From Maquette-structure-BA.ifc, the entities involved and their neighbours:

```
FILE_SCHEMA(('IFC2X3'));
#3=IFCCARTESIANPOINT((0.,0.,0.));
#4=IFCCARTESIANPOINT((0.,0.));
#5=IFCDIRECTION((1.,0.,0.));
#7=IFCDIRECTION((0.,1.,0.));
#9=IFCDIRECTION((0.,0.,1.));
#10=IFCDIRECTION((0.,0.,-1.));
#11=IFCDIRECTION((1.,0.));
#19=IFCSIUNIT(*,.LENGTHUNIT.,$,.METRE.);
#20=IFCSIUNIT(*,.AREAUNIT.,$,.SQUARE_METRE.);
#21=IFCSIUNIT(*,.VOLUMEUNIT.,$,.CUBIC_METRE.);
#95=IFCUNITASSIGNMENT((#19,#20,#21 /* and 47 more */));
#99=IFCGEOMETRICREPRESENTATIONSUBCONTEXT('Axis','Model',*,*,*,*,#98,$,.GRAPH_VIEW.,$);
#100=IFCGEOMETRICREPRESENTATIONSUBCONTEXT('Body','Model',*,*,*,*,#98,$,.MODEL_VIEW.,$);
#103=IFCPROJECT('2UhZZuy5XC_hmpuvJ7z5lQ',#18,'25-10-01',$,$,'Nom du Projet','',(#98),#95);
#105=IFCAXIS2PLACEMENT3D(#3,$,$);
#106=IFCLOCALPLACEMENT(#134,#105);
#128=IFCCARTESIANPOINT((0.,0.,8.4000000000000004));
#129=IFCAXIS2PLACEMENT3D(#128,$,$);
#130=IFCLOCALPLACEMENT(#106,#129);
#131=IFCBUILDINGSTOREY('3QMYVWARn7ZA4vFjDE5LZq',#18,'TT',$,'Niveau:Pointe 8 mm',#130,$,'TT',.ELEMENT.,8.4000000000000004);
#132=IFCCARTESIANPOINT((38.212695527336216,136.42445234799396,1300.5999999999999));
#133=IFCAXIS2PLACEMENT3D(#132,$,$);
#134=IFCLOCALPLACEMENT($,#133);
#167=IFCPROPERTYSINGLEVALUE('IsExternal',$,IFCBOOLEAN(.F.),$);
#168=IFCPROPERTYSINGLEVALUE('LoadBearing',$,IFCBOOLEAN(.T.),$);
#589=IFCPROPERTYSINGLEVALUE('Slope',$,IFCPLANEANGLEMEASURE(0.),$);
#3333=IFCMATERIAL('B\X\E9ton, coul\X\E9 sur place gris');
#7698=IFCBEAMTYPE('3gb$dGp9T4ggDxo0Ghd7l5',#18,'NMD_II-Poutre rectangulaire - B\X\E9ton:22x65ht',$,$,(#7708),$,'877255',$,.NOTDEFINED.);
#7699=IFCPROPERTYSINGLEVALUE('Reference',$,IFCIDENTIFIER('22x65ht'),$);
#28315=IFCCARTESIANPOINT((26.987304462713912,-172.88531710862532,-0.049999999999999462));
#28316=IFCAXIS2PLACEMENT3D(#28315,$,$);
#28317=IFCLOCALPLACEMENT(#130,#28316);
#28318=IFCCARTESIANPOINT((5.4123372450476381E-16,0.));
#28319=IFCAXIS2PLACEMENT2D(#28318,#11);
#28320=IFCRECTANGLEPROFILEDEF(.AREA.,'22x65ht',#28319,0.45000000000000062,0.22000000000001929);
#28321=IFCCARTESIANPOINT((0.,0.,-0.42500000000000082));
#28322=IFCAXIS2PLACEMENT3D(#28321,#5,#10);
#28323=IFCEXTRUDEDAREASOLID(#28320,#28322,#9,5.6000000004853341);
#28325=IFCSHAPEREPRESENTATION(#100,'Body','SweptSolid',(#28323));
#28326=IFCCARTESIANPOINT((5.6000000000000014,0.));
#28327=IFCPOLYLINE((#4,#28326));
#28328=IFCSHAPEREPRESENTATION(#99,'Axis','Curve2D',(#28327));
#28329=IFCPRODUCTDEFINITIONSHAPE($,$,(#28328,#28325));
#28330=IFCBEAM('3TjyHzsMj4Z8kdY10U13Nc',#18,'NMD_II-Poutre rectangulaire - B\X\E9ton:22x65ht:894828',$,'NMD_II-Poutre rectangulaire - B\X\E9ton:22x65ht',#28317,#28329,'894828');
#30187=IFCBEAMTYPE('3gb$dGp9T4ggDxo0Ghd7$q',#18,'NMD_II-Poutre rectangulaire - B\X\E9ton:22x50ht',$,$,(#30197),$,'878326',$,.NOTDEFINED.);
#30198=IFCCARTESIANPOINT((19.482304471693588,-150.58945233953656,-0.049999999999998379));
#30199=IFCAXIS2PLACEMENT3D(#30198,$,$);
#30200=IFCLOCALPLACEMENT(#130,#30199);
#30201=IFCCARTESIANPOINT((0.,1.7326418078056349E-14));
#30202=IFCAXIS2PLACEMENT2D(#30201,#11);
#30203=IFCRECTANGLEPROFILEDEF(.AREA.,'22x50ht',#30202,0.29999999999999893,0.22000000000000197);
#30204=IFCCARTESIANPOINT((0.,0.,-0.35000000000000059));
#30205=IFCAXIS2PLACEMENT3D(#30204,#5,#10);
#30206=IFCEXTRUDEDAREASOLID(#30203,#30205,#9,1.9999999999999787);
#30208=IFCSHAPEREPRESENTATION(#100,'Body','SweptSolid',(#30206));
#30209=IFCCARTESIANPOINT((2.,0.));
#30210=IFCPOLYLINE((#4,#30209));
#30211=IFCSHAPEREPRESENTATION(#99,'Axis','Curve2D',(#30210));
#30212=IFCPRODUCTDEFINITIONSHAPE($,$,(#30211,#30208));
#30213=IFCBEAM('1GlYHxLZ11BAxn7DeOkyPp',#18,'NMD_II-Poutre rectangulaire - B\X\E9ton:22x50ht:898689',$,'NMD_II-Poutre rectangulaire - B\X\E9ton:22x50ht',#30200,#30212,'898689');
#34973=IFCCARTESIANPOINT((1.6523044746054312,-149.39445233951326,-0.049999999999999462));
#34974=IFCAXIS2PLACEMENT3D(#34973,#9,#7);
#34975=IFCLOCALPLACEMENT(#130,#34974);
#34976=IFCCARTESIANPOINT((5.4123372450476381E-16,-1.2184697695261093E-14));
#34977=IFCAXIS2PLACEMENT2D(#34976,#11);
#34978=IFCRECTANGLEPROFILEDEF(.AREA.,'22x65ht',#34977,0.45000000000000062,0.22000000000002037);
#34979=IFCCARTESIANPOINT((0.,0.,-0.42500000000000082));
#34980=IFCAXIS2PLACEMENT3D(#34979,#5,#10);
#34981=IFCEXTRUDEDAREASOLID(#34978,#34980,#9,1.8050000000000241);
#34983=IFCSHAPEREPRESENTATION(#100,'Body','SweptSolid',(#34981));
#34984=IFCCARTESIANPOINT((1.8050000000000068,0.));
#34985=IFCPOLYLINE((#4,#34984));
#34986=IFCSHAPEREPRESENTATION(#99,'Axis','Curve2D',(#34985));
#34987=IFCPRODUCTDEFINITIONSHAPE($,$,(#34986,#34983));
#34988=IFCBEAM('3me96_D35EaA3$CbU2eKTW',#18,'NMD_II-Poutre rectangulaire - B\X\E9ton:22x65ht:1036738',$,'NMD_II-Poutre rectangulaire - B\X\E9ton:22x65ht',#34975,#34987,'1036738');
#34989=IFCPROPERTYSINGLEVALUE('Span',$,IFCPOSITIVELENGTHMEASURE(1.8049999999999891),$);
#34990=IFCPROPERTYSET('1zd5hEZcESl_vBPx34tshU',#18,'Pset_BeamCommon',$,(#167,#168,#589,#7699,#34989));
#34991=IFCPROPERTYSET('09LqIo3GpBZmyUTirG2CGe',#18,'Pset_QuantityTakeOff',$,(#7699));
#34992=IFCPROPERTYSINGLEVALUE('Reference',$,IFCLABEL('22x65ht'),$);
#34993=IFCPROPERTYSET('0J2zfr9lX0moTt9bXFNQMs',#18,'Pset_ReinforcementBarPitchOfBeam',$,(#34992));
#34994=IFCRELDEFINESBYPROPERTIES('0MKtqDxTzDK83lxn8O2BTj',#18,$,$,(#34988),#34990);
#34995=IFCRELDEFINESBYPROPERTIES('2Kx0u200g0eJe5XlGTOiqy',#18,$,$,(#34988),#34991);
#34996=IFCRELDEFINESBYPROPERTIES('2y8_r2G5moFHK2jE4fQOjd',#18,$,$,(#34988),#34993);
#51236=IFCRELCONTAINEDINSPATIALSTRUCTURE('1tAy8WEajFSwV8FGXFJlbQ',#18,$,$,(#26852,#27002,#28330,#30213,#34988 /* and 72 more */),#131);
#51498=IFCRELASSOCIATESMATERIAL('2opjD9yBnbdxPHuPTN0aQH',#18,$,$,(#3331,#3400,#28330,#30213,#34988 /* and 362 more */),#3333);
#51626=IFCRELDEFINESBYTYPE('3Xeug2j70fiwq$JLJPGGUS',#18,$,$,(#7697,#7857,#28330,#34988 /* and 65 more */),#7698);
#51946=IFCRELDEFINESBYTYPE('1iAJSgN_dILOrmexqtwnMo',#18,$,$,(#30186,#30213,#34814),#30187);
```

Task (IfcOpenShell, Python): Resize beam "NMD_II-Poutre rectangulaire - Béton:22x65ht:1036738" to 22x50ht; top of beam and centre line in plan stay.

```python
import ifcopenshell
import ifcopenshell.api.pset
import ifcopenshell.api.type
import ifcopenshell.util.element
import ifcopenshell.util.representation

model = ifcopenshell.open("Maquette-structure-BA.ifc")

member = model.by_id(34988)
source = next(p for p in model.by_type("IfcRectangleProfileDef") if p.ProfileName == "22x50ht")

body = ifcopenshell.util.representation.get_representation(member, "Model", "Body")
solid = body.Items[0]
old_profile = solid.SweptArea

# Copy the section's sizes but keep this member's own profile position.
profile = ifcopenshell.util.element.copy(model, source)
# Profiles are centred, so shift by half the change in depth to hold the top.
shift = (old_profile.XDim - profile.XDim) / 2
x, y = old_profile.Position.Location.Coordinates
up = (-1.0, 0.0)  # upwards, in the solid's own plane
location = model.createIfcCartesianPoint((x + up[0] * shift, y + up[1] * shift))
profile.Position = model.createIfcAxis2Placement2D(location, old_profile.Position.RefDirection)
solid.SweptArea = profile
if not model.get_total_inverses(old_profile):
    ifcopenshell.util.element.remove_deep2(model, old_profile)

new_type = model.by_guid("3gb$dGp9T4ggDxo0Ghd7$q")
ifcopenshell.api.type.assign_type(
    model, related_objects=[member], relating_type=new_type, should_map_representations=False
)
member.Name = member.Name.replace("22x65ht", "22x50ht")
member.ObjectType = "NMD_II-Poutre rectangulaire - Béton:22x50ht"
pset = model.by_id(ifcopenshell.util.element.get_pset(member, "Pset_BeamCommon", should_inherit=False)["id"])
ifcopenshell.api.pset.edit_pset(model, pset=pset, properties={"Reference": "22x50ht"})
pset = model.by_id(ifcopenshell.util.element.get_pset(member, "Pset_QuantityTakeOff", should_inherit=False)["id"])
ifcopenshell.api.pset.edit_pset(model, pset=pset, properties={"Reference": "22x50ht"})
pset = model.by_id(ifcopenshell.util.element.get_pset(member, "Pset_ReinforcementBarPitchOfBeam", should_inherit=False)["id"])
ifcopenshell.api.pset.edit_pset(model, pset=pset, properties={"Reference": "22x50ht"})

print(solid.SweptArea)

model.write("Maquette-structure-BA_edited.ifc")
```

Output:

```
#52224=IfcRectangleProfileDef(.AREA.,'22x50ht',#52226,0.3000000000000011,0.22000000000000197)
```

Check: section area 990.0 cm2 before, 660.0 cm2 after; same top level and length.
